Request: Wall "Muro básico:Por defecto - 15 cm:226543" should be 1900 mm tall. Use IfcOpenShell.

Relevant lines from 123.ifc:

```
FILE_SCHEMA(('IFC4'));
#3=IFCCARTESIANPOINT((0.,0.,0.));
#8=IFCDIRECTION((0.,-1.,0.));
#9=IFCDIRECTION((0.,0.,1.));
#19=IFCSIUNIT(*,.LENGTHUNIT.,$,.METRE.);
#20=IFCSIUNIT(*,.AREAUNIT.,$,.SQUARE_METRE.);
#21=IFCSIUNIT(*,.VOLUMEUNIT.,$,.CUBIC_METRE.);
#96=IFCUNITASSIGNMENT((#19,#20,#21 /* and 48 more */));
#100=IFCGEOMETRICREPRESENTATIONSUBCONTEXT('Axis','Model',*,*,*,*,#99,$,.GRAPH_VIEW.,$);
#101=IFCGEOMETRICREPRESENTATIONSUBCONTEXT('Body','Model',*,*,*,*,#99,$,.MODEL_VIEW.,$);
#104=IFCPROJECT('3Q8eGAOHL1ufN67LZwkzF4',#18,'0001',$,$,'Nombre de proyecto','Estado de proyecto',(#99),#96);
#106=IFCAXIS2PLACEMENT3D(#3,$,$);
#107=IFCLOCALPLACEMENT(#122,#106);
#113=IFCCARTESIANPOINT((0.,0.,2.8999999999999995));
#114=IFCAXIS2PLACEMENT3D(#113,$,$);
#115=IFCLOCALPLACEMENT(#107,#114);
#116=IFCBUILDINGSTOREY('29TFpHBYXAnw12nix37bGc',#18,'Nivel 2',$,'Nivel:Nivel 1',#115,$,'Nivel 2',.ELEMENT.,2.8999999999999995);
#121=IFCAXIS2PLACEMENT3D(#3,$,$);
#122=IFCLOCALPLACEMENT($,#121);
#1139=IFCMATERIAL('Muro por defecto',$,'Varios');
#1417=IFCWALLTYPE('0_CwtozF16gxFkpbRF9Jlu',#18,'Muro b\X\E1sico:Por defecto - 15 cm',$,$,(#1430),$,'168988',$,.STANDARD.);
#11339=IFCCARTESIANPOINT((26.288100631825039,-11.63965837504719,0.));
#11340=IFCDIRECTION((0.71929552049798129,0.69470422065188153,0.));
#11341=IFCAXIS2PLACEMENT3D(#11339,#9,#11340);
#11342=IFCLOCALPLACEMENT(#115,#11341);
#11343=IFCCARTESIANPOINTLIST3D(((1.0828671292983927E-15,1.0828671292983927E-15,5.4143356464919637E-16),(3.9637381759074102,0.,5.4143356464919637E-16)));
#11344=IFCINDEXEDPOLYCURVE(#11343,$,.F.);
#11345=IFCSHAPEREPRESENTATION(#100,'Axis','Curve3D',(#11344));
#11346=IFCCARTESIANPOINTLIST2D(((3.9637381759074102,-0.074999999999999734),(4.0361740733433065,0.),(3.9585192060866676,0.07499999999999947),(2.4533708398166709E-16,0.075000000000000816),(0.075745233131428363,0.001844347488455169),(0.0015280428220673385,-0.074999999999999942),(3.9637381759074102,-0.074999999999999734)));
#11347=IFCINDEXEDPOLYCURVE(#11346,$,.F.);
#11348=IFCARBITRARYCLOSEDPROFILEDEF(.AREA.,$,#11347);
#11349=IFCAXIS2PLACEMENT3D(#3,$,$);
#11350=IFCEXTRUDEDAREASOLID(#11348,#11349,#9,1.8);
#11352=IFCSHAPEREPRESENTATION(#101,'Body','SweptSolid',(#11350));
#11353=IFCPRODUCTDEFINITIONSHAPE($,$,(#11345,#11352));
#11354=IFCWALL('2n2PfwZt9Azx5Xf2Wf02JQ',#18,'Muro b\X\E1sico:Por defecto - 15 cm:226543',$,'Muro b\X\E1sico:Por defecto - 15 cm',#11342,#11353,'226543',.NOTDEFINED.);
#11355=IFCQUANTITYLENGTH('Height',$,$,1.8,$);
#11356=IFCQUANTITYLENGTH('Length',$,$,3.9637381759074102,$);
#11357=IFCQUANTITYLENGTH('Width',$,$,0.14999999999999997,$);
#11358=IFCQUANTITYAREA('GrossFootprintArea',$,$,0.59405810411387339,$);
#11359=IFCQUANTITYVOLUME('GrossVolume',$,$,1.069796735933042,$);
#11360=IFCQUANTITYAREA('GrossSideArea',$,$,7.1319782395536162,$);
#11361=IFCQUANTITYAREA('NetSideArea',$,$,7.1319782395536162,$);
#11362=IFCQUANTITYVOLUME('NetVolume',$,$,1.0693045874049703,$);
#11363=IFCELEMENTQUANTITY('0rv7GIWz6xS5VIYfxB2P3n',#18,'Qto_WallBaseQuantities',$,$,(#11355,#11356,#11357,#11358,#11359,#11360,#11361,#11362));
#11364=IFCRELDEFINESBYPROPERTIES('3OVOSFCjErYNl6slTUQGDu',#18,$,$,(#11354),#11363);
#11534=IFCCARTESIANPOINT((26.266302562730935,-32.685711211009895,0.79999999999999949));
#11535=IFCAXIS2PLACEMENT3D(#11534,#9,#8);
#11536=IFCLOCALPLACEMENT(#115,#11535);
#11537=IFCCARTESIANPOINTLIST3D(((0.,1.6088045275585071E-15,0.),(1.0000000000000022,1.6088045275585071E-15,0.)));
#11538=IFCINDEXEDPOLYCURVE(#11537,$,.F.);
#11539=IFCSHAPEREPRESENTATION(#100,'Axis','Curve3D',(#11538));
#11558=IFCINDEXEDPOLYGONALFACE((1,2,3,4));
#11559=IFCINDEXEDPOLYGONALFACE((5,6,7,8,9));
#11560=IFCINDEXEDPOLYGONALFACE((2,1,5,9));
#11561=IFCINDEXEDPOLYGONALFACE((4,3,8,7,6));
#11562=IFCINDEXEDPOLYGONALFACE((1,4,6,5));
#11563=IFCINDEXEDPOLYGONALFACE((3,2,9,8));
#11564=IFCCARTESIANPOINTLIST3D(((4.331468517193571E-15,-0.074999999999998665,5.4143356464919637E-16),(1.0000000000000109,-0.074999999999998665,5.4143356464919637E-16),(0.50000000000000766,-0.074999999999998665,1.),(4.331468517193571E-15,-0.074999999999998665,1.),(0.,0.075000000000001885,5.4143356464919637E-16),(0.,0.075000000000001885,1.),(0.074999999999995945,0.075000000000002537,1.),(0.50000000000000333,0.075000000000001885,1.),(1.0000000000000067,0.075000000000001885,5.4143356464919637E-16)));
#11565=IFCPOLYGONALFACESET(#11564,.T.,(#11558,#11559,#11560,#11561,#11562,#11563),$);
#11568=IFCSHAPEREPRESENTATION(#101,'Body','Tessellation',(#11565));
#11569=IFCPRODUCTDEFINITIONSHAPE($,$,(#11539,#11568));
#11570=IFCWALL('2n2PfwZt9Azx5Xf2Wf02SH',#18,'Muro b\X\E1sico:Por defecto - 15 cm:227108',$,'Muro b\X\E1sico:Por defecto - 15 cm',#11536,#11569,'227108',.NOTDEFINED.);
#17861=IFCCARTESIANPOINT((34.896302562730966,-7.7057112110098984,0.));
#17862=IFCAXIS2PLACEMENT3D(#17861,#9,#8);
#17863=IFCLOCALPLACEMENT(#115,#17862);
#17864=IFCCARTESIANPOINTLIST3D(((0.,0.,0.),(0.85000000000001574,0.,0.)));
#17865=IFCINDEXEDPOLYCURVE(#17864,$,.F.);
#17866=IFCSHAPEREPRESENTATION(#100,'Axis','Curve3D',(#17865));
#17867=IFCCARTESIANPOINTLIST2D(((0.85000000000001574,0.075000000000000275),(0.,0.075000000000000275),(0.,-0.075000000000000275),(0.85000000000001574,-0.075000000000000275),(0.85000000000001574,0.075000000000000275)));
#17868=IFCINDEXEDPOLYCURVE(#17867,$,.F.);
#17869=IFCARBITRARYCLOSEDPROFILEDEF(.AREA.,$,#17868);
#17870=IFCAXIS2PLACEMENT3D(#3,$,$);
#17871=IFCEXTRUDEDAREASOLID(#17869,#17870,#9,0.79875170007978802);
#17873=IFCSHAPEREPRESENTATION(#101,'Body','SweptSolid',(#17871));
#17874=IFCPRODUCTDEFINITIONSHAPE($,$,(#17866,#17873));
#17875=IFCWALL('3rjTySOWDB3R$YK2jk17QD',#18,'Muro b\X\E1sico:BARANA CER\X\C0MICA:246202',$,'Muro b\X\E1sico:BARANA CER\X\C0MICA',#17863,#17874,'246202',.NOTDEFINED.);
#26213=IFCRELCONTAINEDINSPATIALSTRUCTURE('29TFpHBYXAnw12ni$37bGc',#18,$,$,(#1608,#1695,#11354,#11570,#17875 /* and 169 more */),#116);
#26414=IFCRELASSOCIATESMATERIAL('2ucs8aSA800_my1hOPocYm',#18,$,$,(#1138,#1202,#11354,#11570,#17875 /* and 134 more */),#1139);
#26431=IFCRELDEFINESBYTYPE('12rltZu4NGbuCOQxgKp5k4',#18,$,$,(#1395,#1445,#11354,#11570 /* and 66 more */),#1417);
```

```python
import ifcopenshell
import ifcopenshell.api.pset
import ifcopenshell.geom
import ifcopenshell.util.element
import ifcopenshell.util.representation
import ifcopenshell.util.shape
import ifcopenshell.util.unit

model = ifcopenshell.open("123.ifc")
unit_scale = ifcopenshell.util.unit.calculate_unit_scale(model)
area_scale = ifcopenshell.util.unit.calculate_unit_scale(model, "AREAUNIT")
volume_scale = ifcopenshell.util.unit.calculate_unit_scale(model, "VOLUMEUNIT")
settings = ifcopenshell.geom.settings()


def volume(element):
    """Net volume in cubic metres, openings subtracted."""
    shape = ifcopenshell.geom.create_shape(settings, element)
    return ifcopenshell.util.shape.get_volume(shape.geometry)


wall = model.by_id(11354)
before = volume(wall)

body = ifcopenshell.util.representation.get_representation(wall, "Model", "Body")
solid = body.Items[0]
old_height = solid.Depth
solid.Depth = 1.9 / unit_scale
after = volume(wall)
thickness = 0.15  # wall thickness in metres

# Update the stored height, areas and volumes.
qto = model.by_id(ifcopenshell.util.element.get_pset(wall, "Qto_WallBaseQuantities", should_inherit=False)["id"])
ifcopenshell.api.pset.edit_qto(model, qto=qto, properties={
    "Height": solid.Depth,
    "GrossVolume": ifcopenshell.util.element.get_pset(wall, "Qto_WallBaseQuantities", "GrossVolume") * solid.Depth / old_height,
    "GrossSideArea": ifcopenshell.util.element.get_pset(wall, "Qto_WallBaseQuantities", "GrossSideArea") * solid.Depth / old_height,
    "NetSideArea": after / thickness / area_scale,
    "NetVolume": after / volume_scale,
})

print(f"height {old_height:g} -> {solid.Depth:g}, volume {before:.3f} -> {after:.3f} m3")

model.write("123_edited.ifc")
```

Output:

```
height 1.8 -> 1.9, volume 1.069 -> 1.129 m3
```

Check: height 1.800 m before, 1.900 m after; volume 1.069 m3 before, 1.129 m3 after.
